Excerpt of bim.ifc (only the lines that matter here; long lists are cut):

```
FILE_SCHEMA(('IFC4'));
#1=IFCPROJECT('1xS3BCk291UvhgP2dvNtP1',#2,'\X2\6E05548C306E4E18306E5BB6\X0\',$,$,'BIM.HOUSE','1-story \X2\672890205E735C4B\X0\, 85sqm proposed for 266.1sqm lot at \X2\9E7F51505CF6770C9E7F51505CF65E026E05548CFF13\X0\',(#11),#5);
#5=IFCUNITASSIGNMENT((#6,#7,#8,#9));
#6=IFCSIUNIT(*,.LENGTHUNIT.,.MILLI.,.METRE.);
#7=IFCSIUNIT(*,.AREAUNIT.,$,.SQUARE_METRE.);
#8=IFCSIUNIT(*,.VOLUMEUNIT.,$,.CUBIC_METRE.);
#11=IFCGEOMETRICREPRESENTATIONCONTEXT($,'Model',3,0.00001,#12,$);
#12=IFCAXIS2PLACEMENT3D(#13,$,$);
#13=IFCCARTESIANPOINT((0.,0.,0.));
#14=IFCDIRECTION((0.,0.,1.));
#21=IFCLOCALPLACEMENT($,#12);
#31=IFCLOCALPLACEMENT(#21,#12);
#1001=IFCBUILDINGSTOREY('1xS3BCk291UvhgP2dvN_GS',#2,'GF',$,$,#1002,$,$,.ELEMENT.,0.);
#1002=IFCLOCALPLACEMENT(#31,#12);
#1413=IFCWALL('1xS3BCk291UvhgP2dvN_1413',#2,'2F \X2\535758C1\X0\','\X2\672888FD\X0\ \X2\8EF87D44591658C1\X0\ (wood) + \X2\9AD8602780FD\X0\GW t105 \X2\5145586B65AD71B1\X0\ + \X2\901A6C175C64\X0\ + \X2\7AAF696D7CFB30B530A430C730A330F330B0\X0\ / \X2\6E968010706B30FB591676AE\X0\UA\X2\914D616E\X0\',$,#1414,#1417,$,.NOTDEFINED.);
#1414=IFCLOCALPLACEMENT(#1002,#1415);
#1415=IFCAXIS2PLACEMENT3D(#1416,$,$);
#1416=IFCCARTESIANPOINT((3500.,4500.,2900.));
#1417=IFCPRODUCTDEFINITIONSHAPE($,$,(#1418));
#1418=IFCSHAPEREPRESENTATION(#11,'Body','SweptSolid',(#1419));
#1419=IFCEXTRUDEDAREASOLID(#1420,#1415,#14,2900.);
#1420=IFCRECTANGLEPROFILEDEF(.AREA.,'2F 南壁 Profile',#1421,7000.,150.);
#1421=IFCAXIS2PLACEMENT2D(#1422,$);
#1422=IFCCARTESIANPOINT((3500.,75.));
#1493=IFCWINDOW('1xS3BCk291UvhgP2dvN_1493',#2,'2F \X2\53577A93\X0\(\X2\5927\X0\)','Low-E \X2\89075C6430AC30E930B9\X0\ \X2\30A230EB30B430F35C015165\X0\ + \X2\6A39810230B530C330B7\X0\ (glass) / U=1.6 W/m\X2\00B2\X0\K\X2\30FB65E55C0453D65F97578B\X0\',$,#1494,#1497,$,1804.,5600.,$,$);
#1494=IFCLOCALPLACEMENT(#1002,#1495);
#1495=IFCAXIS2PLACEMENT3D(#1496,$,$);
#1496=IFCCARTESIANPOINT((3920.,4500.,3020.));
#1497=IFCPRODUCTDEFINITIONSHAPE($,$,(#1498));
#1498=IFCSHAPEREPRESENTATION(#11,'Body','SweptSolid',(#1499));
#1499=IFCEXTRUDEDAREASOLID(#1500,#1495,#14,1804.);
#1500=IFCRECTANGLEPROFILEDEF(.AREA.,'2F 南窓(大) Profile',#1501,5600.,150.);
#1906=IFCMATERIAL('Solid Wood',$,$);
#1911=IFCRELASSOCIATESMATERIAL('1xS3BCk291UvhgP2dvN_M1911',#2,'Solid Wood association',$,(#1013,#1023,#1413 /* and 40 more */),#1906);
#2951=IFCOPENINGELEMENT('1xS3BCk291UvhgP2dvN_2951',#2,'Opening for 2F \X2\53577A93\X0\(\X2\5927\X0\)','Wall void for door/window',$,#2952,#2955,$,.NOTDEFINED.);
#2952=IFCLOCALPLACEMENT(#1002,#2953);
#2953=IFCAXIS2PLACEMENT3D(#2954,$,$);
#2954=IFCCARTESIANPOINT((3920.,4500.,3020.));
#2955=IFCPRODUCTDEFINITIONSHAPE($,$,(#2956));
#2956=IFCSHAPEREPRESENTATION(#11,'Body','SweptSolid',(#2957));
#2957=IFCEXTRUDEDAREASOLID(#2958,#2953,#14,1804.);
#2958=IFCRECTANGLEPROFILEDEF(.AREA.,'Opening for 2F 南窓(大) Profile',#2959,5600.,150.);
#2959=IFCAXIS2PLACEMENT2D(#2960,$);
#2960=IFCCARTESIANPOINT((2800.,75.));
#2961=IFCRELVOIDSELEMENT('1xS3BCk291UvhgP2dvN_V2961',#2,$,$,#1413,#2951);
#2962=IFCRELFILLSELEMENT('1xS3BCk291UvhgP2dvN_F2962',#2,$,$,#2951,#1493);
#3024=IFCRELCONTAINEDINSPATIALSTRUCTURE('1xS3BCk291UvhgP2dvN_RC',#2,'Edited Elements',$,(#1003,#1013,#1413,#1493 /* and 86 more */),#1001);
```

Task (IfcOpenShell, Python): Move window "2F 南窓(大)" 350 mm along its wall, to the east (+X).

```python
import ifcopenshell
import ifcopenshell.api.geometry
import ifcopenshell.util.placement
import ifcopenshell.util.unit

model = ifcopenshell.open("bim.ifc")
unit_scale = ifcopenshell.util.unit.calculate_unit_scale(model)

window = model.by_guid("1xS3BCk291UvhgP2dvN_1493")
opening = window.FillsVoids[0].RelatingOpeningElement
wall = opening.VoidsElements[0].RelatingBuildingElement

wall_matrix = ifcopenshell.util.placement.get_local_placement(wall.ObjectPlacement)
shift = wall_matrix[:3, 0] * 0.35 / unit_scale
before = ifcopenshell.util.placement.get_local_placement(window.ObjectPlacement)[:3, 3].copy()

# The window is not placed relative to its opening, so move both.
for product in (opening, window):
    matrix = ifcopenshell.util.placement.get_local_placement(product.ObjectPlacement)
    matrix[:3, 3] += shift
    ifcopenshell.api.geometry.edit_object_placement(model, product=product, matrix=matrix, is_si=False)

after = ifcopenshell.util.placement.get_local_placement(window.ObjectPlacement)[:3, 3]
print("window moved by", (after - before).round(3) + 0.0)

model.write("bim_v2.ifc")
```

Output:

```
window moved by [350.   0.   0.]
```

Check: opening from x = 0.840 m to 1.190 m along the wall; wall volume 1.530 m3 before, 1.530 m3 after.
